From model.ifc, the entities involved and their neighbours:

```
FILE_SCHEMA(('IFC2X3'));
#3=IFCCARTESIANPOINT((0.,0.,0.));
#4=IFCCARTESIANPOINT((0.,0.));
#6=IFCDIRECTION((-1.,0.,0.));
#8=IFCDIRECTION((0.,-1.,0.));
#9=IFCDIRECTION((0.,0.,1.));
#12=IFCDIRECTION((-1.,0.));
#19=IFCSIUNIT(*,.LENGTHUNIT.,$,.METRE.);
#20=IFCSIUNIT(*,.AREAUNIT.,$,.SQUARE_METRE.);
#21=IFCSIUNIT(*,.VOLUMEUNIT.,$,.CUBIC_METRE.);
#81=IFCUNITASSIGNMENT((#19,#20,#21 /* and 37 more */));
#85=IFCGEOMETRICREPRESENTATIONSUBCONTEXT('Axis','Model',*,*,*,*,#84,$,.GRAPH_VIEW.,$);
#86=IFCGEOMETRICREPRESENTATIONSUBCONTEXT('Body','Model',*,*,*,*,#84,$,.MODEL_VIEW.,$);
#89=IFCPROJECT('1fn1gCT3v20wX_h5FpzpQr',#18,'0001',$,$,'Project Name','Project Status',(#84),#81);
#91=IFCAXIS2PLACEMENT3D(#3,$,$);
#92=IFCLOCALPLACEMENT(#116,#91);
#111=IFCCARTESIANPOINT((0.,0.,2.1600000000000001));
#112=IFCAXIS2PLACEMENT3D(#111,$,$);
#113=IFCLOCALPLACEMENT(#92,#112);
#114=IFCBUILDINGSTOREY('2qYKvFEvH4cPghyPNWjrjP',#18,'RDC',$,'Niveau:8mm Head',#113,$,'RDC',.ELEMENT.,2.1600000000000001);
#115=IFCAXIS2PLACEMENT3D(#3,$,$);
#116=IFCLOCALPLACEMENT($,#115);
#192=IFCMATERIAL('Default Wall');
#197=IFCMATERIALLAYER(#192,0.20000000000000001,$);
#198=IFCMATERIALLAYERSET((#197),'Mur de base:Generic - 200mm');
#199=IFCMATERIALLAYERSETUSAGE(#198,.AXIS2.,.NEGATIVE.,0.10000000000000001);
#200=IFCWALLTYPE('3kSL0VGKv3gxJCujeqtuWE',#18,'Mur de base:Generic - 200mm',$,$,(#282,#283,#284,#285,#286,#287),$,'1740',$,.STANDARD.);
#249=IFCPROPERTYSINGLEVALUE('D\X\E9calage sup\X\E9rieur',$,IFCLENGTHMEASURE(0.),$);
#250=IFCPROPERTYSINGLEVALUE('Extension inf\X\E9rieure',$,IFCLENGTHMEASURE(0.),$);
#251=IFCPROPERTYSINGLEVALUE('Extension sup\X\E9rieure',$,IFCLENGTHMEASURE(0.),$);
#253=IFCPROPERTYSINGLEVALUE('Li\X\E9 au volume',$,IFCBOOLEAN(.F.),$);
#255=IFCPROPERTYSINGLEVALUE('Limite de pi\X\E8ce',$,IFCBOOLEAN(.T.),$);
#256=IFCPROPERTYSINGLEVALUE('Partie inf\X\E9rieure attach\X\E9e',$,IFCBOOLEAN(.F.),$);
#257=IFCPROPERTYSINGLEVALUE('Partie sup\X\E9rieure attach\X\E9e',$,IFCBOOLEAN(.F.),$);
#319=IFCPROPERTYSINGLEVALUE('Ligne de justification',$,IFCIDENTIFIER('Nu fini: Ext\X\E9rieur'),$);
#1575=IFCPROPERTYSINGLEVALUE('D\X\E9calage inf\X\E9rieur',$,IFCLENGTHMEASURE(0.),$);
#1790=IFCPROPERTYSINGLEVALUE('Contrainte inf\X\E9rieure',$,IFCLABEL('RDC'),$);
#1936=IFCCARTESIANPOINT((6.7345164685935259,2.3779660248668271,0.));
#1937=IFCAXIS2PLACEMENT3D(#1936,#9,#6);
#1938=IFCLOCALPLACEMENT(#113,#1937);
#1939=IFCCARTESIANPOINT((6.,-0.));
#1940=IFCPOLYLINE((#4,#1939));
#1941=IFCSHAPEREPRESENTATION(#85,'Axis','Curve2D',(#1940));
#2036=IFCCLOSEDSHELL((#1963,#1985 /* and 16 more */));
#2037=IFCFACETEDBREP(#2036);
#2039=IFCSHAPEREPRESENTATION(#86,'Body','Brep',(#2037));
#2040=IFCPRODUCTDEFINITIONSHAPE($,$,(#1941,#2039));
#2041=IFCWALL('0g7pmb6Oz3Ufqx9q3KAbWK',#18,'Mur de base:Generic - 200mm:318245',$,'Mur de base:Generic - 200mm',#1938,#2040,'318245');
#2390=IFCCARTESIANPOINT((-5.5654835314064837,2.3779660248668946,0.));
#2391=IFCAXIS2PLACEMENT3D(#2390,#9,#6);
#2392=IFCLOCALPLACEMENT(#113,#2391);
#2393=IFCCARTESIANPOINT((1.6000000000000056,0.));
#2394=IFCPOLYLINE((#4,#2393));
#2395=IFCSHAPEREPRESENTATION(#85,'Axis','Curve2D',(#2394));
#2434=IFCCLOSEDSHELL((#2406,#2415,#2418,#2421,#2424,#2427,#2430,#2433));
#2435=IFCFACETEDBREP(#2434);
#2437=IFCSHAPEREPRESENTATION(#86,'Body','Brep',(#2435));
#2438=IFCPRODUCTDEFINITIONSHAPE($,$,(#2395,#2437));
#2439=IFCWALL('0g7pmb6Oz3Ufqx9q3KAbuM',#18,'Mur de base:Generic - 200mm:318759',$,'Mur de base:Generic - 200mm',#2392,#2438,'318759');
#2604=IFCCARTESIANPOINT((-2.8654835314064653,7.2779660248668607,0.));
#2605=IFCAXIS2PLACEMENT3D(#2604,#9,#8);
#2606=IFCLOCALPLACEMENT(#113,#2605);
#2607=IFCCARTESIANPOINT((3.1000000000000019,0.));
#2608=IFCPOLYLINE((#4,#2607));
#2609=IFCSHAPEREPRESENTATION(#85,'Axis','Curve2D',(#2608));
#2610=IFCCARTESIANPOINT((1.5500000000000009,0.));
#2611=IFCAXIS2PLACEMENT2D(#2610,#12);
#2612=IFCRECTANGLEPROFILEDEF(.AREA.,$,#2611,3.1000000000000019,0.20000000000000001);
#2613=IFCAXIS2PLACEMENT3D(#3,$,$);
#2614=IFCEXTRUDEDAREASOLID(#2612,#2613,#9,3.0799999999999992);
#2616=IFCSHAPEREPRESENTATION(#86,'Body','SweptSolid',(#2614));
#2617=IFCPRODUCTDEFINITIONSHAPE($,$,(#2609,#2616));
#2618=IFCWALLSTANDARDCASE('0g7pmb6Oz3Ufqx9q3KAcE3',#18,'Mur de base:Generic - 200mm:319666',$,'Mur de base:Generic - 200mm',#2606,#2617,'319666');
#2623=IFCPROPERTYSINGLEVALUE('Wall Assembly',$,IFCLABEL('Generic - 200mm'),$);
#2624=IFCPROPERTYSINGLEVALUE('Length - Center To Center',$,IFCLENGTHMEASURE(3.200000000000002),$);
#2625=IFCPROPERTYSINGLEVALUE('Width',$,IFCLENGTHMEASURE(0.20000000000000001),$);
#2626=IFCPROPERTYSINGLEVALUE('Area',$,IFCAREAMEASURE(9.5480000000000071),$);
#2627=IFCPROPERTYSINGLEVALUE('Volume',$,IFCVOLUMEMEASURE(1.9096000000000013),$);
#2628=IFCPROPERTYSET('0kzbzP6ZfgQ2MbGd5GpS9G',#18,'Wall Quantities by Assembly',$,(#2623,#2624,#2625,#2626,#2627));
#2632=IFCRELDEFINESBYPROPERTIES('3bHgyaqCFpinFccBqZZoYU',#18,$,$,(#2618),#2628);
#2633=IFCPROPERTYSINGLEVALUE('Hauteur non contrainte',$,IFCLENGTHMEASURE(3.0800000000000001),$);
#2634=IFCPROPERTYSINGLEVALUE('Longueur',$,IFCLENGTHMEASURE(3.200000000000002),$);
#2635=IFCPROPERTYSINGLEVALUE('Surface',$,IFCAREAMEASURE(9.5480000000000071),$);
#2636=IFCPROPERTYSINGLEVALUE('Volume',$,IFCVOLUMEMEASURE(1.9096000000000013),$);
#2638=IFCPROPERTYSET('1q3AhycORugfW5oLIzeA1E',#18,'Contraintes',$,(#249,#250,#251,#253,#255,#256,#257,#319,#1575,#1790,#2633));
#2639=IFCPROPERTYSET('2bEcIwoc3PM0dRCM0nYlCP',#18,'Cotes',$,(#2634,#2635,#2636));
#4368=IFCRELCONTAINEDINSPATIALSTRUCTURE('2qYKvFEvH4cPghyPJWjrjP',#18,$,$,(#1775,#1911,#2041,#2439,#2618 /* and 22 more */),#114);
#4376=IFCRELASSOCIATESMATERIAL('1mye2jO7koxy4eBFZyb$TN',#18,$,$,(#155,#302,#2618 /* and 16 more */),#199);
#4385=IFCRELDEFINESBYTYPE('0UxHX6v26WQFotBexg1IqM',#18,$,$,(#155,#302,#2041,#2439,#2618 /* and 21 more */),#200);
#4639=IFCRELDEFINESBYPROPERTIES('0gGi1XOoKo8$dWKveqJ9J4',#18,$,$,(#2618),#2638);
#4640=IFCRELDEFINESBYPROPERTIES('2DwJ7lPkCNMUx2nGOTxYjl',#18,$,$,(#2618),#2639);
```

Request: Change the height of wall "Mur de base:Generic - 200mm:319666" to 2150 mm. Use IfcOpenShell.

```python
import ifcopenshell
import ifcopenshell.api.pset
import ifcopenshell.geom
import ifcopenshell.util.element
import ifcopenshell.util.representation
import ifcopenshell.util.shape
import ifcopenshell.util.unit

model = ifcopenshell.open("model.ifc")
area_scale = ifcopenshell.util.unit.calculate_unit_scale(model, "AREAUNIT")
volume_scale = ifcopenshell.util.unit.calculate_unit_scale(model, "VOLUMEUNIT")
settings = ifcopenshell.geom.settings()


def volume(element):
    """Net volume in cubic metres, openings subtracted."""
    shape = ifcopenshell.geom.create_shape(settings, element)
    return ifcopenshell.util.shape.get_volume(shape.geometry)


wall = model.by_guid("0g7pmb6Oz3Ufqx9q3KAcE3")
before = volume(wall)

body = ifcopenshell.util.representation.get_representation(wall, "Model", "Body")
solid = body.Items[0]
old_height = solid.Depth
solid.Depth = 2.15
after = volume(wall)
thickness = 0.2  # wall thickness in metres

# Update the stored height, areas and volumes.
pset = model.by_id(ifcopenshell.util.element.get_pset(wall, "Wall Quantities by Assembly", should_inherit=False)["id"])
ifcopenshell.api.pset.edit_pset(model, pset=pset, properties={
    "Area": model.create_entity("IfcAreaMeasure", after / thickness / area_scale),
    "Volume": model.create_entity("IfcVolumeMeasure", after / volume_scale),
})
pset = model.by_id(ifcopenshell.util.element.get_pset(wall, "Contraintes", should_inherit=False)["id"])
ifcopenshell.api.pset.edit_pset(model, pset=pset, properties={
    "Hauteur non contrainte": model.create_entity("IfcLengthMeasure", solid.Depth),
})
pset = model.by_id(ifcopenshell.util.element.get_pset(wall, "Cotes", should_inherit=False)["id"])
ifcopenshell.api.pset.edit_pset(model, pset=pset, properties={
    "Surface": model.create_entity("IfcAreaMeasure", after / thickness / area_scale),
    "Volume": model.create_entity("IfcVolumeMeasure", after / volume_scale),
})

print(f"height {old_height:g} -> {solid.Depth:g}, volume {before:.3f} -> {after:.3f} m3")

model.write("model_edited.ifc")
```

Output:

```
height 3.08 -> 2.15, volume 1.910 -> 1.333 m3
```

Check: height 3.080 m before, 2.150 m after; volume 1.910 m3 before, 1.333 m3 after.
